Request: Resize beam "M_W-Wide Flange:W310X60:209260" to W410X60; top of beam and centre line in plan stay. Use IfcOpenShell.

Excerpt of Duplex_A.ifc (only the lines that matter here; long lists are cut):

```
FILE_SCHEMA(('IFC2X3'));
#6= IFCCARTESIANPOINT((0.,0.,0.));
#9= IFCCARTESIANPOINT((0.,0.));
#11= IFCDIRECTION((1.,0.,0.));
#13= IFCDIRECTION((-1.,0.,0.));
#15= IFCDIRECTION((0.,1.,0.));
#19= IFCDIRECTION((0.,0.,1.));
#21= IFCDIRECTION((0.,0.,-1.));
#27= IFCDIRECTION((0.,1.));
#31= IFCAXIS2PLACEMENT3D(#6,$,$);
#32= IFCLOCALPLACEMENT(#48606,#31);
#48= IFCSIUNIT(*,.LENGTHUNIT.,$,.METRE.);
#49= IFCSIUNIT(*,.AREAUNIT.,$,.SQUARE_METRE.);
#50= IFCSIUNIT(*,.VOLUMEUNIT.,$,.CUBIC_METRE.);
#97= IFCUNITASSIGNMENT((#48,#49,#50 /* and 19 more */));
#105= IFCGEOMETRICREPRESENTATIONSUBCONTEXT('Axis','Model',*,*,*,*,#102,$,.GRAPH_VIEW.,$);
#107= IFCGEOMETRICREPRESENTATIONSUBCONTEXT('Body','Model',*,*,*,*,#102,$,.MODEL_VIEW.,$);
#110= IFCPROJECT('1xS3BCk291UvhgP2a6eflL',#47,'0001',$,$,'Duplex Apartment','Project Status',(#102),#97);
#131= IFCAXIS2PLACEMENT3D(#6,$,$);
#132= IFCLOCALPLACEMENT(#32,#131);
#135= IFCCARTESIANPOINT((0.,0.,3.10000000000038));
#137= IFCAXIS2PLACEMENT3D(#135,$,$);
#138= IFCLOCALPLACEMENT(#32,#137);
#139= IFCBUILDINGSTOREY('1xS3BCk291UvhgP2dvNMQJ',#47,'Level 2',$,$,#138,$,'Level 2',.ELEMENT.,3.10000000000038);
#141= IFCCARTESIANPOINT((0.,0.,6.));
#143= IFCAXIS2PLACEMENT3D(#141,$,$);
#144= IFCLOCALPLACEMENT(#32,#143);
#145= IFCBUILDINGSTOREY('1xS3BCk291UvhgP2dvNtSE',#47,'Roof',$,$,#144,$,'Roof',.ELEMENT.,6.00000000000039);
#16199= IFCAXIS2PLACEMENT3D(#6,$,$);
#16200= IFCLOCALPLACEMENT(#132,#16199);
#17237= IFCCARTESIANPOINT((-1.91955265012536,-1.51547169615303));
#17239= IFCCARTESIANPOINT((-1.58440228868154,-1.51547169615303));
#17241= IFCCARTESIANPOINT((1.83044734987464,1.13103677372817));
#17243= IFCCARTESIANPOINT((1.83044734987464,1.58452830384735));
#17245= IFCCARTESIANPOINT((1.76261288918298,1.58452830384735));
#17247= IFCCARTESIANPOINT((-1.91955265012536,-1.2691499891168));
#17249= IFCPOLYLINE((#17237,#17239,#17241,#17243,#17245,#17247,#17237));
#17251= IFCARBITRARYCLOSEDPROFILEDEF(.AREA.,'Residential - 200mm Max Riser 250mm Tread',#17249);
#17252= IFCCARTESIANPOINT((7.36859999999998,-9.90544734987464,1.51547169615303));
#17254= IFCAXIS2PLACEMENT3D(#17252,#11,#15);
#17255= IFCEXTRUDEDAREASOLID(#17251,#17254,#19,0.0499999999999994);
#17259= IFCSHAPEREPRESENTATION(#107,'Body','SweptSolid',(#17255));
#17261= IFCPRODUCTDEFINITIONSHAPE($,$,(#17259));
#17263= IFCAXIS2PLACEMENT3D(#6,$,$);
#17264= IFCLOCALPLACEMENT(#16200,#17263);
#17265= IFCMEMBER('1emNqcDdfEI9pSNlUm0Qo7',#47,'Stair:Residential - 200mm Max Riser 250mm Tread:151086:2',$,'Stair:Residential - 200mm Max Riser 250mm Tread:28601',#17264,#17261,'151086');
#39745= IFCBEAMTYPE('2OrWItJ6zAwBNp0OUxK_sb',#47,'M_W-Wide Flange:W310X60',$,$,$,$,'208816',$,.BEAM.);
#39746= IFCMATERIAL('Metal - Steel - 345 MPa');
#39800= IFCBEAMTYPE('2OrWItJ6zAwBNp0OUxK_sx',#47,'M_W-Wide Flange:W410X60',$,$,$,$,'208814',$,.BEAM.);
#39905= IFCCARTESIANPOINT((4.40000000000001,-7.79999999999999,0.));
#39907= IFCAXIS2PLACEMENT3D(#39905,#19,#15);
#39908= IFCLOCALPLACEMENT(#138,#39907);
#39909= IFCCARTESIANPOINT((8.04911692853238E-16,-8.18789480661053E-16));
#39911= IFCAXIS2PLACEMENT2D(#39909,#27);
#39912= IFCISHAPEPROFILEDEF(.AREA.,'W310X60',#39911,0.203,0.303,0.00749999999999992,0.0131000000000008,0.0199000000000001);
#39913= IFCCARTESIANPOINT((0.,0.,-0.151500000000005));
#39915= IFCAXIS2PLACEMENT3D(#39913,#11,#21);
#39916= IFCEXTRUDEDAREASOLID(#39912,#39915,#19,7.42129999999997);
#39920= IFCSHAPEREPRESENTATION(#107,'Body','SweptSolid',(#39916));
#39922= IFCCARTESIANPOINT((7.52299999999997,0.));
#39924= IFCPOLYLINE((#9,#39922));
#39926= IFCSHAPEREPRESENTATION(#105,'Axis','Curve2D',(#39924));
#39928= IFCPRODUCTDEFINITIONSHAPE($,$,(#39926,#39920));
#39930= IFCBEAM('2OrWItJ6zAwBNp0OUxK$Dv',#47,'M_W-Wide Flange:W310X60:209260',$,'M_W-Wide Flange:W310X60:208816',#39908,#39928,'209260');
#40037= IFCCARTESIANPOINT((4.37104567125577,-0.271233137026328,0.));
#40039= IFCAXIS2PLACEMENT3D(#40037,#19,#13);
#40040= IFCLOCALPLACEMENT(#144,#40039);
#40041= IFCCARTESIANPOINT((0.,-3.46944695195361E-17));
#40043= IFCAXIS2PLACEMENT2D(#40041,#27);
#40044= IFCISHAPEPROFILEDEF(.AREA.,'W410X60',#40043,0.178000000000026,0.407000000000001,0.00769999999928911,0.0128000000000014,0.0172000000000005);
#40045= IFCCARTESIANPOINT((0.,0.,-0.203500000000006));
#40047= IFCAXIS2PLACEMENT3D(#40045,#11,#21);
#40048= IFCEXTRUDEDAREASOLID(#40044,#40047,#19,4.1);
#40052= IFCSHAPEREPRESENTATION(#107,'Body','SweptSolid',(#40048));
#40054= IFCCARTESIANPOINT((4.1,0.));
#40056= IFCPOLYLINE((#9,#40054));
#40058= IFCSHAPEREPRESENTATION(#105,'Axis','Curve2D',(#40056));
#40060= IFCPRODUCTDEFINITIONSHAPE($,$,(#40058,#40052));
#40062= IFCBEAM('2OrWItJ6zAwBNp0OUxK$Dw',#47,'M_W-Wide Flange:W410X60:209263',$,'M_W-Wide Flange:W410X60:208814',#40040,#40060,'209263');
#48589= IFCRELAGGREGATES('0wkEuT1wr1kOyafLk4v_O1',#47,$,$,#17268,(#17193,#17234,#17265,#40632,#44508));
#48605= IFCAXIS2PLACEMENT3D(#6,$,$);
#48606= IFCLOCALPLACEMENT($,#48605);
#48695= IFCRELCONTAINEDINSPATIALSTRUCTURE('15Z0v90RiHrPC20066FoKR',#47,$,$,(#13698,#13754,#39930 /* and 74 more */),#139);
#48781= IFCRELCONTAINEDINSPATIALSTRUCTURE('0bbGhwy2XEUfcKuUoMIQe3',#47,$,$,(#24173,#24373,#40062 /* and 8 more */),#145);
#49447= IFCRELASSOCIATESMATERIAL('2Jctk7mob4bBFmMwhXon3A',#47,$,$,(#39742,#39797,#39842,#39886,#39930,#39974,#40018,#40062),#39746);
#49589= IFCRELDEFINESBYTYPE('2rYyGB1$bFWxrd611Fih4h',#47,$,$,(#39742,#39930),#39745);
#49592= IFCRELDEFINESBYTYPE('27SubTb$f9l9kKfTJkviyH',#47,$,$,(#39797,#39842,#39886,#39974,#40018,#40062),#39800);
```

```python
import ifcopenshell
import ifcopenshell.api.type
import ifcopenshell.util.element
import ifcopenshell.util.representation

model = ifcopenshell.open("Duplex_A.ifc")

member = model.by_guid("2OrWItJ6zAwBNp0OUxK$Dv")
source = next(p for p in model.by_type("IfcIShapeProfileDef") if p.ProfileName == "W410X60")

body = ifcopenshell.util.representation.get_representation(member, "Model", "Body")
solid = body.Items[0]
old_profile = solid.SweptArea

# Copy the section's sizes but keep this member's own profile position.
profile = ifcopenshell.util.element.copy(model, source)
# Profiles are centred, so shift by half the change in depth to hold the top.
shift = (old_profile.OverallDepth - profile.OverallDepth) / 2
x, y = old_profile.Position.Location.Coordinates
up = (-1.0, 0.0)  # upwards, in the solid's own plane
location = model.createIfcCartesianPoint((x + up[0] * shift, y + up[1] * shift))
profile.Position = model.createIfcAxis2Placement2D(location, old_profile.Position.RefDirection)
solid.SweptArea = profile
if not model.get_total_inverses(old_profile):
    ifcopenshell.util.element.remove_deep2(model, old_profile)

new_type = model.by_id(39800)
ifcopenshell.api.type.assign_type(
    model, related_objects=[member], relating_type=new_type, should_map_representations=False
)
member.Name = member.Name.replace("W310X60", "W410X60")
member.ObjectType = "M_W-Wide Flange:W410X60:208816"

print(solid.SweptArea)

model.write("Duplex_A_edited.ifc")
```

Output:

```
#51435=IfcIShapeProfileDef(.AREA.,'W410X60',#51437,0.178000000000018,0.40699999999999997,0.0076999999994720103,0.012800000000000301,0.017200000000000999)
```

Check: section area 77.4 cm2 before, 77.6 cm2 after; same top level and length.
